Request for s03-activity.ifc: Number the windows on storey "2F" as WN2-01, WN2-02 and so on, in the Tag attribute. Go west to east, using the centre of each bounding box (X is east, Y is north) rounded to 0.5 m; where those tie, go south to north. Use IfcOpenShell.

First a look at what the model holds.

```python
import ifcopenshell
import ifcopenshell.util.element
import ifcopenshell.util.placement

model = ifcopenshell.open("s03-activity.ifc")
print(model.schema)
storey = next(s for s in model.by_type("IfcBuildingStorey") if s.Name == "2F")
windows = [e for e in ifcopenshell.util.element.get_decomposition(storey) if e.is_a("IfcWindow")]
for e in sorted(windows, key=lambda e: e.id()):
    origin = ifcopenshell.util.placement.get_local_placement(e.ObjectPlacement)[:3, 3]
    print(e.id(), e.Tag, e.Name, origin.round(2) + 0.0, sep=" | ")
```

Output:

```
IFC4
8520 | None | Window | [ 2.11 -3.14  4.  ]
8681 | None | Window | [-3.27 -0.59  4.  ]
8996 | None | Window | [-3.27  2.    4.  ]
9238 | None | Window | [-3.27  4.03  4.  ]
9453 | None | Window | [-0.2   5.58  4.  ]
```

```python
import ifcopenshell
import ifcopenshell.geom
import ifcopenshell.util.element
import ifcopenshell.util.shape

model = ifcopenshell.open("s03-activity.ifc")
settings = ifcopenshell.geom.settings()
settings.set("use-world-coords", True)


def centre(element):
    shape = ifcopenshell.geom.create_shape(settings, element)
    return ifcopenshell.util.shape.get_bbox_centroid(shape.geometry)


storey = next(s for s in model.by_type("IfcBuildingStorey") if s.Name == "2F")
windows = [e for e in ifcopenshell.util.element.get_decomposition(storey) if e.is_a("IfcWindow")]

# Insertion points can sit at a corner or the storey origin, so sort by the geometry (in metres).
centres = {e: centre(e) for e in windows}
windows.sort(key=lambda e: (round(centres[e][0] / 0.5), centres[e][1]))

for i, e in enumerate(windows, start=1):
    number = f"WN2-{i:02d}"
    e.Tag = number
    print(e.id(), number)

model.write("s03-activity_rev.ifc")
```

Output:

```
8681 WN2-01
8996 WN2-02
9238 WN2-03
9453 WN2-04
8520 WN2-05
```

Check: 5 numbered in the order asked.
